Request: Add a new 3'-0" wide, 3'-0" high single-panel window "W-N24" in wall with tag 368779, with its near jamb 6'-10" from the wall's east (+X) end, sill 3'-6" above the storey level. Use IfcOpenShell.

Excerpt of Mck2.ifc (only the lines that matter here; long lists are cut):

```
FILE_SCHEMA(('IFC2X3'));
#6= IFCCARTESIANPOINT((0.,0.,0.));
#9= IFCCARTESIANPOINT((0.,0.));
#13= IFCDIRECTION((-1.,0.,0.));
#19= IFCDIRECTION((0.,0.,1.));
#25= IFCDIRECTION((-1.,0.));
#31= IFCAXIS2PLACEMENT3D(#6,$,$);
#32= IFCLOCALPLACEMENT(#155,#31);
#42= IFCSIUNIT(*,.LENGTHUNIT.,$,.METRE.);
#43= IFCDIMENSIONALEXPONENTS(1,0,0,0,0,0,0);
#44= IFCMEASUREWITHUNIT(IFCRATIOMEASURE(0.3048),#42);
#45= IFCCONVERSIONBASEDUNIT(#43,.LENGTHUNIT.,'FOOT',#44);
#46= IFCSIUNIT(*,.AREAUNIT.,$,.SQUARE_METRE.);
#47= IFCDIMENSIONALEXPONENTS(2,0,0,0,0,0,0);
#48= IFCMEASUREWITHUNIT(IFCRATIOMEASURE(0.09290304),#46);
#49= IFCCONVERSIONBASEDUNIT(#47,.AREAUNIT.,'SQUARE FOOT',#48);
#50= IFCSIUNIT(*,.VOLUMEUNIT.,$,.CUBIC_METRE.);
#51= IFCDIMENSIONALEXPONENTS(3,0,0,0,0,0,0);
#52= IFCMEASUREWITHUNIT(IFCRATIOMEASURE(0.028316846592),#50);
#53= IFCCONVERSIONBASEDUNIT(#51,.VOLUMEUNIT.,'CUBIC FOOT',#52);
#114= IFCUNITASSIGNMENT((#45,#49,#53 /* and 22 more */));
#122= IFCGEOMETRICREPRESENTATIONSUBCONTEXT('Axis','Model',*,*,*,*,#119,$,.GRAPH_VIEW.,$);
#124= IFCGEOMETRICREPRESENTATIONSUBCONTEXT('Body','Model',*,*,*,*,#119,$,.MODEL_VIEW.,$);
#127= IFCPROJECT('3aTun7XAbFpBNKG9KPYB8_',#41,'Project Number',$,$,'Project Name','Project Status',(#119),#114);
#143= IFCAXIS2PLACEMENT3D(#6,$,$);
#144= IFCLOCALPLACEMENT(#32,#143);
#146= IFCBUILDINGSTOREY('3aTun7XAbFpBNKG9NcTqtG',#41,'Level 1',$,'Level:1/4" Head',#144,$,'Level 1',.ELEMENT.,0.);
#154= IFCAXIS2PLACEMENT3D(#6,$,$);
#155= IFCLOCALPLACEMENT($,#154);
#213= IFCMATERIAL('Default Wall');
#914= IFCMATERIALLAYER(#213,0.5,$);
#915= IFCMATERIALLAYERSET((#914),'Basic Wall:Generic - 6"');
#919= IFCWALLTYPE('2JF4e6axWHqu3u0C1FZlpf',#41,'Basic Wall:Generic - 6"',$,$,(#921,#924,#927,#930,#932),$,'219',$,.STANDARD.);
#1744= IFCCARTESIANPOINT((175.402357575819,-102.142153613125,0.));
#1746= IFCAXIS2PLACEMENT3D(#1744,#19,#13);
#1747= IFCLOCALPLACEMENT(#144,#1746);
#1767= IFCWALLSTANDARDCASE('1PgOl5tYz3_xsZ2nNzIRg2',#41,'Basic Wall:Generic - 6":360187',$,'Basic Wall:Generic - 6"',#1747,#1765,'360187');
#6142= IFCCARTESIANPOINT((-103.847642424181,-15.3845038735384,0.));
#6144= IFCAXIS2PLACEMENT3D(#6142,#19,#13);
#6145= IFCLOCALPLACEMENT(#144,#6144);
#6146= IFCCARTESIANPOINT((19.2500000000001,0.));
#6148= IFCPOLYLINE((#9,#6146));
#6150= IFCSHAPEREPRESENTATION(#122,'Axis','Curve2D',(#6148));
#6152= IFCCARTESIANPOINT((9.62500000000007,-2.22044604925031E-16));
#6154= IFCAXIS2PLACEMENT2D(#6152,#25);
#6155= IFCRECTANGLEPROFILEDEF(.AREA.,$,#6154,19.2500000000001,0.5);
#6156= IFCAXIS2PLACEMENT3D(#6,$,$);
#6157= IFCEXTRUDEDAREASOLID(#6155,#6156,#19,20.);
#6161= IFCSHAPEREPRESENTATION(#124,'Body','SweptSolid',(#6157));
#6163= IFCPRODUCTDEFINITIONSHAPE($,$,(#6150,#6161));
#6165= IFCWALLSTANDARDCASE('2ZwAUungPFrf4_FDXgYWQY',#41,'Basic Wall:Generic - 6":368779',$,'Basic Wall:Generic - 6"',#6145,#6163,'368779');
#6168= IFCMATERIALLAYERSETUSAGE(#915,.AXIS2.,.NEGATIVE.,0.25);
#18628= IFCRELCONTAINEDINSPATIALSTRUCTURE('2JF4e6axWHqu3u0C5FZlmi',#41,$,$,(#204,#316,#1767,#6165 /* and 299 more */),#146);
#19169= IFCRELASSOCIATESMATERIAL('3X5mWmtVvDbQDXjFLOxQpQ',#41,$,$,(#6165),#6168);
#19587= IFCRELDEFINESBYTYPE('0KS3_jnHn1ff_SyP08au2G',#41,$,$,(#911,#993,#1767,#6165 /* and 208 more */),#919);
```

```python
import numpy as np
import ifcopenshell
import ifcopenshell.api.feature
import ifcopenshell.api.geometry
import ifcopenshell.api.root
import ifcopenshell.api.spatial
import ifcopenshell.api.type
import ifcopenshell.geom
import ifcopenshell.util.element
import ifcopenshell.util.placement
import ifcopenshell.util.representation
import ifcopenshell.util.shape
import ifcopenshell.util.unit

model = ifcopenshell.open("Mck2.ifc")
unit_scale = ifcopenshell.util.unit.calculate_unit_scale(model)
settings = ifcopenshell.geom.settings()


def volume(element):
    """Net volume in cubic metres, openings subtracted."""
    shape = ifcopenshell.geom.create_shape(settings, element)
    return ifcopenshell.util.shape.get_volume(shape.geometry)


wall = model.by_guid("2ZwAUungPFrf4_FDXgYWQY")
storey = ifcopenshell.util.element.get_container(wall, ifc_class="IfcBuildingStorey")
context = ifcopenshell.util.representation.get_context(model, "Model", "Body", "MODEL_VIEW")
before = volume(wall)

width, height, from_end, sill = 0.9144, 0.9144, 2.0828, 1.0668  # metres

# The wall runs along its own X axis, and the end named is its -X end.
wall_shape = ifcopenshell.geom.create_shape(settings, wall)
x, y, z = ifcopenshell.util.shape.get_vertices(wall_shape.geometry).T
start = x.min() + from_end
face, thickness = float(y.min()), float(y.max() - y.min())
wall_matrix = ifcopenshell.util.placement.get_local_placement(wall.ObjectPlacement)
level = ifcopenshell.util.placement.get_local_placement(storey.ObjectPlacement)[2, 3]


def in_wall(x, y):
    """Placement at x, y metres in the wall's axes, at sill height."""
    matrix = wall_matrix.copy()
    matrix[:, 3] = wall_matrix @ np.array([x / unit_scale, y / unit_scale, 0.0, 1.0])
    matrix[2, 3] = level + sill / unit_scale
    return matrix


# Opening: a box that overshoots both wall faces by 50 mm.
opening = ifcopenshell.api.root.create_entity(model, ifc_class="IfcOpeningElement")
box = ifcopenshell.api.geometry.add_wall_representation(
    model, context=context, length=width, height=height, thickness=thickness + 0.1
)
ifcopenshell.api.geometry.assign_representation(model, product=opening, representation=box)
ifcopenshell.api.geometry.edit_object_placement(model, product=opening, matrix=in_wall(start, face - 0.05), is_si=False)
ifcopenshell.api.feature.add_feature(model, feature=opening, element=wall)

window = ifcopenshell.api.root.create_entity(model, ifc_class="IfcWindow", name="W-N24")
window.OverallWidth, window.OverallHeight = width / unit_scale, height / unit_scale
body = ifcopenshell.api.geometry.add_window_representation(
    model,
    context=context,
    overall_width=window.OverallWidth,
    overall_height=window.OverallHeight,
    partition_type="SINGLE_PANEL",
)
ifcopenshell.api.geometry.assign_representation(model, product=window, representation=body)
ifcopenshell.api.spatial.assign_container(model, products=[window], relating_structure=storey)
fills = ifcopenshell.api.feature.add_filling(model, opening=opening, element=window)
fills.OwnerHistory = window.OwnerHistory  # required in IFC2X3

# IFC2X3 keeps the operation on the window style.
style = ifcopenshell.api.root.create_entity(model, ifc_class="IfcWindowStyle", name="W-N24")
style.OperationType, style.ConstructionType = "SINGLE_PANEL", "NOTDEFINED"
style.ParameterTakesPrecedence = style.Sizeable = False
ifcopenshell.api.type.assign_type(model, related_objects=[window], relating_type=style)

# Centre the window in the wall's thickness.
ifcopenshell.api.geometry.edit_object_placement(model, product=window, matrix=in_wall(start, face), is_si=False)
window_shape = ifcopenshell.geom.create_shape(settings, window)
depth = ifcopenshell.util.shape.get_vertices(window_shape.geometry)[:, 1]
offset = face + thickness / 2 - (depth.min() + depth.max()) / 2
ifcopenshell.api.geometry.edit_object_placement(model, product=window, matrix=in_wall(start, offset), is_si=False)

after = volume(wall)

print(f"wall volume {before:.3f} -> {after:.3f} m3")

model.write("Mck2-out.ifc")
```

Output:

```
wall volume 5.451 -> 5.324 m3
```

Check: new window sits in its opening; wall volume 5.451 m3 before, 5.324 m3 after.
